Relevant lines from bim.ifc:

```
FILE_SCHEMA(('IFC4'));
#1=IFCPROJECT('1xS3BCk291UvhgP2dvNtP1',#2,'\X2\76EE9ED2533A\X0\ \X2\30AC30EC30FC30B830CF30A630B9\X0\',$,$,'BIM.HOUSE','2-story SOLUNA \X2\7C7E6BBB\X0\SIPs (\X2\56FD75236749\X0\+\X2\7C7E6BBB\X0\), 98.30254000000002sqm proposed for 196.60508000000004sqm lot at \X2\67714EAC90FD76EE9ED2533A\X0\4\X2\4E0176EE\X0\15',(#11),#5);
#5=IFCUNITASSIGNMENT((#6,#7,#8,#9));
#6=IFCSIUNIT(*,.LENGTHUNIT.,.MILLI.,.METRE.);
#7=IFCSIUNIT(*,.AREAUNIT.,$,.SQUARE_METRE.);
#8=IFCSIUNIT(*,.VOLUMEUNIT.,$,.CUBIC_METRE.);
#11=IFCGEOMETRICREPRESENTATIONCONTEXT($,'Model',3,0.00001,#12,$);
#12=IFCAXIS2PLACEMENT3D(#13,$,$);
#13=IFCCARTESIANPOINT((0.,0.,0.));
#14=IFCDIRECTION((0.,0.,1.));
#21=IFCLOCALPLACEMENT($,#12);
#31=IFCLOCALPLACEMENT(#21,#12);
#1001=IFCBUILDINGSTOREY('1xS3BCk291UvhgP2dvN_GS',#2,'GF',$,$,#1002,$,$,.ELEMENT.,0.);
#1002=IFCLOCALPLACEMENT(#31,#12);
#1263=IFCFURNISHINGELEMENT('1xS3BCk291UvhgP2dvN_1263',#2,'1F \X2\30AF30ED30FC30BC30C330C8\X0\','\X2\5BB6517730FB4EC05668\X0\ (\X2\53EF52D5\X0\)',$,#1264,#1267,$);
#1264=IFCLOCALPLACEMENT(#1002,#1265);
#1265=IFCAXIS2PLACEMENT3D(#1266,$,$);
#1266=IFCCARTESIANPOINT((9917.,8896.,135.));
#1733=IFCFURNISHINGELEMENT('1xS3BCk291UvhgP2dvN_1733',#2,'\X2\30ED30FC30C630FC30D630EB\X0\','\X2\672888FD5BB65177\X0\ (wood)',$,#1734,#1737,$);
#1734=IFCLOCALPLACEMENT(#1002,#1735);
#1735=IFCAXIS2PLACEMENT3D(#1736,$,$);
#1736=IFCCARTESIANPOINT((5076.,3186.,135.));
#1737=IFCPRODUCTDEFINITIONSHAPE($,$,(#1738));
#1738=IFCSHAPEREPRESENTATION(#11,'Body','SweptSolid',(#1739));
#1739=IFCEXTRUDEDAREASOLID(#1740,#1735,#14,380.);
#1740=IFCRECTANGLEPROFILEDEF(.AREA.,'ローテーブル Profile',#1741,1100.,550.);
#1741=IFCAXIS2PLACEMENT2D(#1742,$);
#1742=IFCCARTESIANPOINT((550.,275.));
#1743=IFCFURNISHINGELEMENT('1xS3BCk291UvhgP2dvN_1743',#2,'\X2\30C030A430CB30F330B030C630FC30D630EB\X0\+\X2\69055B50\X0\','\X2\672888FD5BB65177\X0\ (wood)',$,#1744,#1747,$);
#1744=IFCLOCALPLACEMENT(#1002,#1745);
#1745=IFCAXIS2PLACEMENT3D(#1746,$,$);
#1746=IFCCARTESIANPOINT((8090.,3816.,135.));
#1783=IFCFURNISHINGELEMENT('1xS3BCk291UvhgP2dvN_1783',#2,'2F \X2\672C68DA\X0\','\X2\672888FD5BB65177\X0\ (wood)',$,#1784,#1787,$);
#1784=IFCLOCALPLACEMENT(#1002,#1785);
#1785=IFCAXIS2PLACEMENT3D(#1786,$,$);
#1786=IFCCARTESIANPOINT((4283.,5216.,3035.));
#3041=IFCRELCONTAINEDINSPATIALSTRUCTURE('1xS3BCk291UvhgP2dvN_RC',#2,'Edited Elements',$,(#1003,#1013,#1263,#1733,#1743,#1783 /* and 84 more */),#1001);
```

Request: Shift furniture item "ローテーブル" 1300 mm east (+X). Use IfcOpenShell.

```python
import ifcopenshell
import ifcopenshell.api.geometry
import ifcopenshell.util.placement
import ifcopenshell.util.unit

model = ifcopenshell.open("bim.ifc")
unit_scale = ifcopenshell.util.unit.calculate_unit_scale(model)

item = model.by_guid("1xS3BCk291UvhgP2dvN_1733")
matrix = ifcopenshell.util.placement.get_local_placement(item.ObjectPlacement)
matrix[0, 3] += 1.3 / unit_scale
ifcopenshell.api.geometry.edit_object_placement(model, product=item, matrix=matrix, is_si=False)

print(ifcopenshell.util.placement.get_local_placement(item.ObjectPlacement).round(3) + 0.0)

model.write("bim-out.ifc")
```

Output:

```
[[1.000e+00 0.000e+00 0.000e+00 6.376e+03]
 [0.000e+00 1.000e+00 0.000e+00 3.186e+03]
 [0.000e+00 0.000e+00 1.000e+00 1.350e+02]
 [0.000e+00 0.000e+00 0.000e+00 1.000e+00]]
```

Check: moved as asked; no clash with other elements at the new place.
